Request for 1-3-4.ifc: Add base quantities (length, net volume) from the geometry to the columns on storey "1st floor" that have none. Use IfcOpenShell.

First a look at what the model holds.

```python
import ifcopenshell
import ifcopenshell.util.element
import ifcopenshell.util.unit

model = ifcopenshell.open("1-3-4.ifc")
print(model.schema)
for unit_type in ("LENGTHUNIT", "AREAUNIT", "VOLUMEUNIT"):
    print(unit_type, ifcopenshell.util.unit.calculate_unit_scale(model, unit_type))
storey = next(s for s in model.by_type("IfcBuildingStorey") if s.Name == "1st floor")
columns = [e for e in ifcopenshell.util.element.get_decomposition(storey) if e.is_a("IfcColumn")]
for e in sorted(columns, key=lambda e: e.id()):
    print(e.id(), e.is_a(), e.Name, list(ifcopenshell.util.element.get_psets(e, qtos_only=True)), sep=" | ")
```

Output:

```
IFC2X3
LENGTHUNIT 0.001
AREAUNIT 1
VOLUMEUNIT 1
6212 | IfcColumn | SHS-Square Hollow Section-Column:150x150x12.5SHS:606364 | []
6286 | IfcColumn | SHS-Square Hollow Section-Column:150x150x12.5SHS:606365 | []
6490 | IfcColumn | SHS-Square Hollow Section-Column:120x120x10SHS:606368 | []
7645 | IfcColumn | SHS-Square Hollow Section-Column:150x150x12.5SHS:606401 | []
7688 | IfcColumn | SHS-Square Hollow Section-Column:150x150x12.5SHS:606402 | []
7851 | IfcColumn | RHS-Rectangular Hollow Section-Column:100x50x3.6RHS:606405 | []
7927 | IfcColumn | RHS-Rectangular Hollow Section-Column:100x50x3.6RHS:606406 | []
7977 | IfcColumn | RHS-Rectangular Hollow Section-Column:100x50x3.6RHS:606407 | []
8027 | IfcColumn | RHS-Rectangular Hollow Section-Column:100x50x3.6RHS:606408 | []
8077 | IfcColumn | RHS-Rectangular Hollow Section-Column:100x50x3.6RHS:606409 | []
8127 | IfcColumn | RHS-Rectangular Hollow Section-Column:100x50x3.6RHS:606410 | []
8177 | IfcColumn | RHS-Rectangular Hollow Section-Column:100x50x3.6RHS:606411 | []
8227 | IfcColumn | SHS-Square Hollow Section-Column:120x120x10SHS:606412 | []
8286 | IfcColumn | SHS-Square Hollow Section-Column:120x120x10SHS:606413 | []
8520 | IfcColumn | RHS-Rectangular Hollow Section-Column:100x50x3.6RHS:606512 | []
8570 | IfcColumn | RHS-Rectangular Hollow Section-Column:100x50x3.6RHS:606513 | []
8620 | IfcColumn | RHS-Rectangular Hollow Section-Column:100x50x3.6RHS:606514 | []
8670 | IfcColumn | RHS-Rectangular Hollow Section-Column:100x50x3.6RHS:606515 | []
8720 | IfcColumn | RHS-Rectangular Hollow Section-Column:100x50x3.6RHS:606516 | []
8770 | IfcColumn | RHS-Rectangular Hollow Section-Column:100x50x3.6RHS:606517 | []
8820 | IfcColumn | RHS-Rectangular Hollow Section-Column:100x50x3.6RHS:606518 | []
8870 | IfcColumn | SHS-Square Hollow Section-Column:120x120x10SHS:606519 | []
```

```python
import ifcopenshell
import ifcopenshell.api.pset
import ifcopenshell.geom
import ifcopenshell.util.element
import ifcopenshell.util.shape
import ifcopenshell.util.unit

model = ifcopenshell.open("1-3-4.ifc")
unit_scale = ifcopenshell.util.unit.calculate_unit_scale(model)
volume_scale = ifcopenshell.util.unit.calculate_unit_scale(model, "VOLUMEUNIT")
settings = ifcopenshell.geom.settings()

storey = next(s for s in model.by_type("IfcBuildingStorey") if s.Name == "1st floor")
columns = [e for e in ifcopenshell.util.element.get_decomposition(storey) if e.is_a("IfcColumn")]

for e in sorted(columns, key=lambda e: e.id()):
    if ifcopenshell.util.element.get_psets(e, qtos_only=True, should_inherit=False):
        continue
    # Geometry comes back in metres, in the element's own axes.
    shape = ifcopenshell.geom.create_shape(settings, e)
    values = {
        "Length": ifcopenshell.util.shape.get_z(shape.geometry) / unit_scale,
        "NetVolume": ifcopenshell.util.shape.get_volume(shape.geometry) / volume_scale,
    }
    qto = ifcopenshell.api.pset.add_qto(model, product=e, name="BaseQuantities")
    ifcopenshell.api.pset.edit_qto(model, qto=qto, properties=values)
    print(e.id(), {k: round(v, 3) for k, v in values.items()})

model.write("1-3-4_updated.ifc")
```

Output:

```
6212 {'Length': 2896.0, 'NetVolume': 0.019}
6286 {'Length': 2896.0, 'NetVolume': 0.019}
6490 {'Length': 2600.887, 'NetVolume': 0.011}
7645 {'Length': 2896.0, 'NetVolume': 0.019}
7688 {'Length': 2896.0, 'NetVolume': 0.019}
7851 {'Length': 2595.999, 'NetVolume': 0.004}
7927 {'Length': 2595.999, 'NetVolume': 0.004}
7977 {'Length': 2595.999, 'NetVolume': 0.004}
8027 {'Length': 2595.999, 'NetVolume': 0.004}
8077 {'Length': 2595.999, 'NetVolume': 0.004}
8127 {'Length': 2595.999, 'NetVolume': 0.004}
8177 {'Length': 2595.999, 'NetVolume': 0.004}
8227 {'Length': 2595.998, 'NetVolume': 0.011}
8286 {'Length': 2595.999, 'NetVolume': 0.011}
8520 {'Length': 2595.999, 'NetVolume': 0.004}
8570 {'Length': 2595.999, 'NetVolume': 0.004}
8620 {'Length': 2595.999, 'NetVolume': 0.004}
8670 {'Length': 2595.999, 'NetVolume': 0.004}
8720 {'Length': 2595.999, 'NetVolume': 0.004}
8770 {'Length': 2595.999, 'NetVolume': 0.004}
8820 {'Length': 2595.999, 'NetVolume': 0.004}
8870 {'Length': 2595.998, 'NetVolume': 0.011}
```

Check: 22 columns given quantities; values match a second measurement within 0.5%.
